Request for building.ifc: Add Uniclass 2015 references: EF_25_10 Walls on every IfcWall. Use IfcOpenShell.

First a look at what the model holds.

```python
import ifcopenshell

model = ifcopenshell.open("building.ifc")
print(model.schema)
print("classifications:", [c.Name for c in model.by_type("IfcClassification")])
for ifc_class in ("IfcDoor", "IfcRoof", "IfcStair", "IfcWall", "IfcWindow"):
    print(ifc_class, len(model.by_type(ifc_class)))
```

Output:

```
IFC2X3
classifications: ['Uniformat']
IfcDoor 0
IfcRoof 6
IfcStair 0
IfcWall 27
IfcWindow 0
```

```python
import ifcopenshell
import ifcopenshell.api.classification

model = ifcopenshell.open("building.ifc")

# IFC2X3 requires Source and Edition and has no link from the project to the system.
system = model.create_entity("IfcClassification", Source="NBS", Edition="2015", Name="Uniclass 2015")

codes = {
    "IfcWall": ("EF_25_10", "Walls"),
}
for ifc_class, (code, name) in codes.items():
    products = model.by_type(ifc_class)
    ifcopenshell.api.classification.add_reference(
        model, products=products, classification=system, identification=code, name=name
    )
    print(code, len(products))

model.write("building_v2.ifc")
```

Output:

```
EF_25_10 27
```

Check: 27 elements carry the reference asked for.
